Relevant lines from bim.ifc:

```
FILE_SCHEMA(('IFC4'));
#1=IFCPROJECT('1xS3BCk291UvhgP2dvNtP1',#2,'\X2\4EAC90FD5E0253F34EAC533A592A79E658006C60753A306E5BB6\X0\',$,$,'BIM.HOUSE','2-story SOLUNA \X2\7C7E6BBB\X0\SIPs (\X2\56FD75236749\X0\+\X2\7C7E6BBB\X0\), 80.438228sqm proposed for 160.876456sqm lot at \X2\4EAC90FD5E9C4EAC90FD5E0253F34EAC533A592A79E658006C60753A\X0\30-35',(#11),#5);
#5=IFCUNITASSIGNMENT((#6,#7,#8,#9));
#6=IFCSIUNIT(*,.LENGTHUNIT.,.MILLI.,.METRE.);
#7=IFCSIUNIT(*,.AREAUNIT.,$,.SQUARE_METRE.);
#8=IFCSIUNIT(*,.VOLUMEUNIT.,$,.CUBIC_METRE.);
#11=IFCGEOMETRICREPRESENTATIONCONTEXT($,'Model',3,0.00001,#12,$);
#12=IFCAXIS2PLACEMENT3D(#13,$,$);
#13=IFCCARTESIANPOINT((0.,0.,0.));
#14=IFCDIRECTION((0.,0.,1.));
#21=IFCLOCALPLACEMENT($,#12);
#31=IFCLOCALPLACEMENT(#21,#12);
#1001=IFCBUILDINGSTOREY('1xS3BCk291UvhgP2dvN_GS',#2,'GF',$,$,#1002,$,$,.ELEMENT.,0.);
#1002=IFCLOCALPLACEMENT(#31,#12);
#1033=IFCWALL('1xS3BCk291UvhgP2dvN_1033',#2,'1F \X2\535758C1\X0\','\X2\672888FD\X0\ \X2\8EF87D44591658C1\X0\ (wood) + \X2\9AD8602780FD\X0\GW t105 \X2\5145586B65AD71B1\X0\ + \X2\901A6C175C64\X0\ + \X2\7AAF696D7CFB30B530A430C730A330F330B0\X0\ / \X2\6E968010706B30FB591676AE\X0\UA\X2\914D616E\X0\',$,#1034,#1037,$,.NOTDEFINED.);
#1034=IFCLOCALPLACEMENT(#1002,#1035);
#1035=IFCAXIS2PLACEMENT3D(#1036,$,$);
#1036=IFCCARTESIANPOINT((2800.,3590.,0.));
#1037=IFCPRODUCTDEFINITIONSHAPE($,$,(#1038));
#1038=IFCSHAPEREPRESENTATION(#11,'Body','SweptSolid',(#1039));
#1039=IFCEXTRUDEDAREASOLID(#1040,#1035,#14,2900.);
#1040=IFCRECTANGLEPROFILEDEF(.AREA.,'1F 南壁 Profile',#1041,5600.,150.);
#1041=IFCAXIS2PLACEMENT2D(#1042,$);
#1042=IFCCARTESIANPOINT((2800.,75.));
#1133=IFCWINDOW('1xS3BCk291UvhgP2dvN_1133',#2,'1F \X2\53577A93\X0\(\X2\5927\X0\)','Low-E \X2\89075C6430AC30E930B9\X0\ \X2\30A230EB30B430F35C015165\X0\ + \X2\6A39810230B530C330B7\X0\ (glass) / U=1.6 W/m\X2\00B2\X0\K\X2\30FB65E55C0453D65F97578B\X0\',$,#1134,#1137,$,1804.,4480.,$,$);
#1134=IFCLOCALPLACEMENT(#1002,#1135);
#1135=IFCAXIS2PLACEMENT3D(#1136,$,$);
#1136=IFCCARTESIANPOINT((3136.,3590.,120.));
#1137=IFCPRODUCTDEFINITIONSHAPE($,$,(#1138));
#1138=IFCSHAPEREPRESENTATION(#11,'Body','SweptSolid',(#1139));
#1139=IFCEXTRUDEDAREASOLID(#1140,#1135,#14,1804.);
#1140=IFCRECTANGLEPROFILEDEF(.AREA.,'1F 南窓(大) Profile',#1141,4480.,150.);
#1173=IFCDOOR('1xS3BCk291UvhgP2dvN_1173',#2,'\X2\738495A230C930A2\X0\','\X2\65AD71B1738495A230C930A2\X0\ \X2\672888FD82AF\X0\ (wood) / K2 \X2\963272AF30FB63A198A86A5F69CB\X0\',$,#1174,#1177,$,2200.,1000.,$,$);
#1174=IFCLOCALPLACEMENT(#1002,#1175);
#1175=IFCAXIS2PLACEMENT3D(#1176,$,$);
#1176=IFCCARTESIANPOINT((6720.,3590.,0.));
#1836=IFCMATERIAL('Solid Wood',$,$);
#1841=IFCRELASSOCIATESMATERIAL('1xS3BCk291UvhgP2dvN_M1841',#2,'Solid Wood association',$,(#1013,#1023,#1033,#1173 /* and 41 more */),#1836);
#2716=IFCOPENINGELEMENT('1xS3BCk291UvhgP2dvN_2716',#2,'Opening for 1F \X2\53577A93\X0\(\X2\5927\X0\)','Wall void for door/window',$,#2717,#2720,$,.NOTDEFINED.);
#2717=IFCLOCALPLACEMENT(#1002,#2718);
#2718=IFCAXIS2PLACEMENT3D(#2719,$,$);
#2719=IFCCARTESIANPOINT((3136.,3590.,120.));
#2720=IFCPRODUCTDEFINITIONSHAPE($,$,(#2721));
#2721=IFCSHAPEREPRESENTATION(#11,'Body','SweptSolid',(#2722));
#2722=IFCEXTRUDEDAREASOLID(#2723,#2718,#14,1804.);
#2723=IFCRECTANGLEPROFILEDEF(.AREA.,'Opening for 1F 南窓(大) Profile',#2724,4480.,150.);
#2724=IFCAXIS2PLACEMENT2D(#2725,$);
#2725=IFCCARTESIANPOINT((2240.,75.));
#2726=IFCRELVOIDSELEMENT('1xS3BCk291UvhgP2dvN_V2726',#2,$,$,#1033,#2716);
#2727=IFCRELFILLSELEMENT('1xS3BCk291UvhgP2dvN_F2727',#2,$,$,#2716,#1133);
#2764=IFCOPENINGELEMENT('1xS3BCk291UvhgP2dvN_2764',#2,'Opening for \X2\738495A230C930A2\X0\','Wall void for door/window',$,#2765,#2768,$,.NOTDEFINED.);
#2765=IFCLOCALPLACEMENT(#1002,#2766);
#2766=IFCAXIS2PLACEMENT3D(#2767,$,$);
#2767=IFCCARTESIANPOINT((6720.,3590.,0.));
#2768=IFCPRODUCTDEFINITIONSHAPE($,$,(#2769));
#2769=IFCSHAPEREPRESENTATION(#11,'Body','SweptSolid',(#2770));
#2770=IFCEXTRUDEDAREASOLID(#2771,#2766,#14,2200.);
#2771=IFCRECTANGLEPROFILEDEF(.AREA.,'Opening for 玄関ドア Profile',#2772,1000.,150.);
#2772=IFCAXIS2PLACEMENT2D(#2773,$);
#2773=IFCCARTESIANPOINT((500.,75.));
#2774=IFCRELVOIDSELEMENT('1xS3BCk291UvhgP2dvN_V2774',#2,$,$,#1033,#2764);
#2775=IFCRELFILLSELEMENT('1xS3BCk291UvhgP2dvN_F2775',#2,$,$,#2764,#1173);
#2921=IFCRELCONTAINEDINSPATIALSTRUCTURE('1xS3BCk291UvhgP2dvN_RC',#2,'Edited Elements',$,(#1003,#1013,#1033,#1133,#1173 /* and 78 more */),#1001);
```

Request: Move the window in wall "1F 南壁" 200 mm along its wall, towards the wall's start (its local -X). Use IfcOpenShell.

```python
import ifcopenshell
import ifcopenshell.api.geometry
import ifcopenshell.util.placement

model = ifcopenshell.open("bim.ifc")

window = model.by_guid("1xS3BCk291UvhgP2dvN_1133")
opening = window.FillsVoids[0].RelatingOpeningElement
wall = opening.VoidsElements[0].RelatingBuildingElement

wall_matrix = ifcopenshell.util.placement.get_local_placement(wall.ObjectPlacement)
shift = wall_matrix[:3, 0] * -200.0
before = ifcopenshell.util.placement.get_local_placement(window.ObjectPlacement)[:3, 3].copy()

# The window is not placed relative to its opening, so move both.
for product in (opening, window):
    matrix = ifcopenshell.util.placement.get_local_placement(product.ObjectPlacement)
    matrix[:3, 3] += shift
    ifcopenshell.api.geometry.edit_object_placement(model, product=product, matrix=matrix, is_si=False)

after = ifcopenshell.util.placement.get_local_placement(window.ObjectPlacement)[:3, 3]
print("window moved by", (after - before).round(3) + 0.0)

model.write("bim_edited.ifc")
```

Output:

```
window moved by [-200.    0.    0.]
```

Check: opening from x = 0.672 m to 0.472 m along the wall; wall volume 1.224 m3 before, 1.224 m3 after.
